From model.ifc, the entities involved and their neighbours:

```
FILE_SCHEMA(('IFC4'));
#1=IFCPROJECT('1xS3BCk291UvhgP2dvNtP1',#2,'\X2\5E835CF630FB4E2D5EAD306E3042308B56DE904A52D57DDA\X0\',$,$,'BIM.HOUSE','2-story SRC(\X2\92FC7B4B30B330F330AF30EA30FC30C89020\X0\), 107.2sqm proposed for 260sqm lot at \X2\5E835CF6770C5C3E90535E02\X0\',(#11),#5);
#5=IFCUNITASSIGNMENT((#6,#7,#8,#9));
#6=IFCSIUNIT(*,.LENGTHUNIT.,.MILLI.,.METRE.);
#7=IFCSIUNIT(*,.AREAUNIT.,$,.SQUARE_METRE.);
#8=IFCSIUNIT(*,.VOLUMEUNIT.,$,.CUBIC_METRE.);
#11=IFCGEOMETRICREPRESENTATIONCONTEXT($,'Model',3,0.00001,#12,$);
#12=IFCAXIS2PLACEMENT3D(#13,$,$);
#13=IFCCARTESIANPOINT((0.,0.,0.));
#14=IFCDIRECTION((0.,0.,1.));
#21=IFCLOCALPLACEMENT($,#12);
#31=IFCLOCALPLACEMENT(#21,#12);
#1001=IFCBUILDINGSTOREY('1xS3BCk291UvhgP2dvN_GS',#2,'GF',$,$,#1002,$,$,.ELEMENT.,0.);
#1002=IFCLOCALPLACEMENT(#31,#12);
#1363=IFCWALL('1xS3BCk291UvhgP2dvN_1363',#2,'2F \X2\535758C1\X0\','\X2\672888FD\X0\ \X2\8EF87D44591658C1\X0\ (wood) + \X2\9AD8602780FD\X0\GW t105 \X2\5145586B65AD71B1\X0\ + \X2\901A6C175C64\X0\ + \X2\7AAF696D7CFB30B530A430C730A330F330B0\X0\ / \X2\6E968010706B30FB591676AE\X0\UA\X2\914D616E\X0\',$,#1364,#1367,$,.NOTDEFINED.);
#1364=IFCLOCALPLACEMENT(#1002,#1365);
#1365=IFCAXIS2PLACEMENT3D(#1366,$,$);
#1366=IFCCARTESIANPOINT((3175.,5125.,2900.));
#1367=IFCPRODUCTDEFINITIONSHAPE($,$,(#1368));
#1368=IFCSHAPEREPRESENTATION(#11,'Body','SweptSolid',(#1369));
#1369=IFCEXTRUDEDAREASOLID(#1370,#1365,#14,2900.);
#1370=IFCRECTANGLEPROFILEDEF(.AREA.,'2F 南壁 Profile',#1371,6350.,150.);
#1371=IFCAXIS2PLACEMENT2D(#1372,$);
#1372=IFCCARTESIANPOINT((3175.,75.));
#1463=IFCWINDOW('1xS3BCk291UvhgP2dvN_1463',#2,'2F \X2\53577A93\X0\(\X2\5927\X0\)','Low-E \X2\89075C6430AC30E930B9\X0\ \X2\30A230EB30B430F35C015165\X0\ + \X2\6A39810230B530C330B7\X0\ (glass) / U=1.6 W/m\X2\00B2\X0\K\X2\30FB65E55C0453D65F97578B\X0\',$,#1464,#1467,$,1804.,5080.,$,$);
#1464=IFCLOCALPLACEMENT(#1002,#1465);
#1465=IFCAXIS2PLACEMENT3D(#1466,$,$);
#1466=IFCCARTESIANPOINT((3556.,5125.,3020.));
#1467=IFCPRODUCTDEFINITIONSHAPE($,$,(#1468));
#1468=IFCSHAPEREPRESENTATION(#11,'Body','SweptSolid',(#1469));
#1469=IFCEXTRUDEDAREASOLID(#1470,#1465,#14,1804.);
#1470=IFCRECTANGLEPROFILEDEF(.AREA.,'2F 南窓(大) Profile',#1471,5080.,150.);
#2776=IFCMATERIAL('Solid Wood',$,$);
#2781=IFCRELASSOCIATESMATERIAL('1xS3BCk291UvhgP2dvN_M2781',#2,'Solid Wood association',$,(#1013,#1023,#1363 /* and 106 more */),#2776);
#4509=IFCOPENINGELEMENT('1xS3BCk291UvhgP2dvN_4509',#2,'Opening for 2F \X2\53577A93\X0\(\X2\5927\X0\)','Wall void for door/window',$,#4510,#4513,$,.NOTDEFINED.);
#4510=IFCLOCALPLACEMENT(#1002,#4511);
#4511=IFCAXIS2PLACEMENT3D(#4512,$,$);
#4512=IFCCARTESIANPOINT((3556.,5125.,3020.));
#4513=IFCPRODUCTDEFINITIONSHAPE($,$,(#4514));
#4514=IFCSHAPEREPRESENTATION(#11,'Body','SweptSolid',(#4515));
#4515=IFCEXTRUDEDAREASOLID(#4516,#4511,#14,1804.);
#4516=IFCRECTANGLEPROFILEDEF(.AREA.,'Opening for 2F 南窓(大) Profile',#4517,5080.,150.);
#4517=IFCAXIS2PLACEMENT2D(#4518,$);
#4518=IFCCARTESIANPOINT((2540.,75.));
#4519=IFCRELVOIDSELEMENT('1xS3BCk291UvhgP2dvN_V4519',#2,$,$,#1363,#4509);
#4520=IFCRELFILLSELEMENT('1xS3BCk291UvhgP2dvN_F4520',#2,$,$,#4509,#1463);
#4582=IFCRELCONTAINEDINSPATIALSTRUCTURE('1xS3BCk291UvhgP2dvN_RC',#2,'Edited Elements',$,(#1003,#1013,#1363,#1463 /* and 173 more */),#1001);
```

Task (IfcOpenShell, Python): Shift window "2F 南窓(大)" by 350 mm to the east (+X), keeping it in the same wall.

```python
import ifcopenshell
import ifcopenshell.api.geometry
import ifcopenshell.util.placement

model = ifcopenshell.open("model.ifc")

window = model.by_guid("1xS3BCk291UvhgP2dvN_1463")
opening = window.FillsVoids[0].RelatingOpeningElement
wall = opening.VoidsElements[0].RelatingBuildingElement

wall_matrix = ifcopenshell.util.placement.get_local_placement(wall.ObjectPlacement)
shift = wall_matrix[:3, 0] * 350.0
before = ifcopenshell.util.placement.get_local_placement(window.ObjectPlacement)[:3, 3].copy()

# The window is not placed relative to its opening, so move both.
for product in (opening, window):
    matrix = ifcopenshell.util.placement.get_local_placement(product.ObjectPlacement)
    matrix[:3, 3] += shift
    ifcopenshell.api.geometry.edit_object_placement(model, product=product, matrix=matrix, is_si=False)

after = ifcopenshell.util.placement.get_local_placement(window.ObjectPlacement)[:3, 3]
print("window moved by", (after - before).round(3) + 0.0)

model.write("model-out.ifc")
```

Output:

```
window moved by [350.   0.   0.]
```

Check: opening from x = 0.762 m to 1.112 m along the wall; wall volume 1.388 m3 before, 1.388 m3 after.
